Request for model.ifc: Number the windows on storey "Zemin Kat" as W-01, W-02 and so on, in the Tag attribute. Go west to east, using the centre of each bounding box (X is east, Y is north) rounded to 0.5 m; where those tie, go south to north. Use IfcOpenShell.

First a look at what the model holds.

```python
import ifcopenshell
import ifcopenshell.util.element
import ifcopenshell.util.placement

model = ifcopenshell.open("model.ifc")
print(model.schema)
storey = next(s for s in model.by_type("IfcBuildingStorey") if s.Name == "Zemin Kat")
windows = [e for e in ifcopenshell.util.element.get_decomposition(storey) if e.is_a("IfcWindow")]
for e in sorted(windows, key=lambda e: e.id()):
    origin = ifcopenshell.util.placement.get_local_placement(e.ObjectPlacement)[:3, 3]
    print(e.id(), e.Tag, e.Name, origin.round(2) + 0.0, sep=" | ")
```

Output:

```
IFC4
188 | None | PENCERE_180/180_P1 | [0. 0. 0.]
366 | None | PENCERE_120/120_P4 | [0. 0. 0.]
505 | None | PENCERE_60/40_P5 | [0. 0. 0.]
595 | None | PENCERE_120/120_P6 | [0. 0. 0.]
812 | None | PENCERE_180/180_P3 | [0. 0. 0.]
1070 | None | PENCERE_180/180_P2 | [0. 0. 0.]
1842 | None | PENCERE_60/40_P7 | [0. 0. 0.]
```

```python
import ifcopenshell
import ifcopenshell.geom
import ifcopenshell.util.element
import ifcopenshell.util.shape

model = ifcopenshell.open("model.ifc")
settings = ifcopenshell.geom.settings()
settings.set("use-world-coords", True)


def centre(element):
    shape = ifcopenshell.geom.create_shape(settings, element)
    return ifcopenshell.util.shape.get_bbox_centroid(shape.geometry)


storey = next(s for s in model.by_type("IfcBuildingStorey") if s.Name == "Zemin Kat")
windows = [e for e in ifcopenshell.util.element.get_decomposition(storey) if e.is_a("IfcWindow")]

# Insertion points can sit at a corner or the storey origin, so sort by the geometry (in metres).
centres = {e: centre(e) for e in windows}
windows.sort(key=lambda e: (round(centres[e][0] / 0.5), centres[e][1]))

for i, e in enumerate(windows, start=1):
    number = f"W-{i:02d}"
    e.Tag = number
    print(e.id(), number)

model.write("model_edited.ifc")
```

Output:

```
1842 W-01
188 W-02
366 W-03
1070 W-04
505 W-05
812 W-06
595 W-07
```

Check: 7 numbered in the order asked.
